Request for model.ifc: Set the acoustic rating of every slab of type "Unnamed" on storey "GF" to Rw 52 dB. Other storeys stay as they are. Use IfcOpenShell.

First a look at what the model holds.

```python
import ifcopenshell
import ifcopenshell.util.element

model = ifcopenshell.open("model.ifc")
print(model.schema)
storey = next(s for s in model.by_type("IfcBuildingStorey") if s.Name == "GF")
slabs = [e for e in ifcopenshell.util.element.get_decomposition(storey) if e.is_a("IfcSlab")]
seen = {}
for e in slabs:
    element_type = ifcopenshell.util.element.get_type(e)
    key = (element_type.Name if element_type != e and element_type else None, ifcopenshell.util.element.get_pset(e, "Pset_SlabCommon", "AcousticRating"))
    seen[key] = seen.get(key, 0) + 1
for (name, value), count in sorted(seen.items(), key=str):
    print(count, "x", name, "|", value)
```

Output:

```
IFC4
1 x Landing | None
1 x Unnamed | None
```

```python
import ifcopenshell
import ifcopenshell.api.pset
import ifcopenshell.util.element

model = ifcopenshell.open("model.ifc")

storey = next(s for s in model.by_type("IfcBuildingStorey") if s.Name == "GF")
slabs = [e for e in ifcopenshell.util.element.get_decomposition(storey) if e.is_a("IfcSlab")]

count = 0
for e in slabs:
    element_type = ifcopenshell.util.element.get_type(e)
    if element_type in (None, e) or element_type.Name != "Unnamed":
        continue
    # add_pset returns the element's existing set when there is one.
    pset = ifcopenshell.api.pset.add_pset(model, product=e, name="Pset_SlabCommon")
    ifcopenshell.api.pset.edit_pset(model, pset=pset, properties={"AcousticRating": "Rw 52 dB"})
    count += 1

print(count, "slabs updated")

model.write("model_rev.ifc")
```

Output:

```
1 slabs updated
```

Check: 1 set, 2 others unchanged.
